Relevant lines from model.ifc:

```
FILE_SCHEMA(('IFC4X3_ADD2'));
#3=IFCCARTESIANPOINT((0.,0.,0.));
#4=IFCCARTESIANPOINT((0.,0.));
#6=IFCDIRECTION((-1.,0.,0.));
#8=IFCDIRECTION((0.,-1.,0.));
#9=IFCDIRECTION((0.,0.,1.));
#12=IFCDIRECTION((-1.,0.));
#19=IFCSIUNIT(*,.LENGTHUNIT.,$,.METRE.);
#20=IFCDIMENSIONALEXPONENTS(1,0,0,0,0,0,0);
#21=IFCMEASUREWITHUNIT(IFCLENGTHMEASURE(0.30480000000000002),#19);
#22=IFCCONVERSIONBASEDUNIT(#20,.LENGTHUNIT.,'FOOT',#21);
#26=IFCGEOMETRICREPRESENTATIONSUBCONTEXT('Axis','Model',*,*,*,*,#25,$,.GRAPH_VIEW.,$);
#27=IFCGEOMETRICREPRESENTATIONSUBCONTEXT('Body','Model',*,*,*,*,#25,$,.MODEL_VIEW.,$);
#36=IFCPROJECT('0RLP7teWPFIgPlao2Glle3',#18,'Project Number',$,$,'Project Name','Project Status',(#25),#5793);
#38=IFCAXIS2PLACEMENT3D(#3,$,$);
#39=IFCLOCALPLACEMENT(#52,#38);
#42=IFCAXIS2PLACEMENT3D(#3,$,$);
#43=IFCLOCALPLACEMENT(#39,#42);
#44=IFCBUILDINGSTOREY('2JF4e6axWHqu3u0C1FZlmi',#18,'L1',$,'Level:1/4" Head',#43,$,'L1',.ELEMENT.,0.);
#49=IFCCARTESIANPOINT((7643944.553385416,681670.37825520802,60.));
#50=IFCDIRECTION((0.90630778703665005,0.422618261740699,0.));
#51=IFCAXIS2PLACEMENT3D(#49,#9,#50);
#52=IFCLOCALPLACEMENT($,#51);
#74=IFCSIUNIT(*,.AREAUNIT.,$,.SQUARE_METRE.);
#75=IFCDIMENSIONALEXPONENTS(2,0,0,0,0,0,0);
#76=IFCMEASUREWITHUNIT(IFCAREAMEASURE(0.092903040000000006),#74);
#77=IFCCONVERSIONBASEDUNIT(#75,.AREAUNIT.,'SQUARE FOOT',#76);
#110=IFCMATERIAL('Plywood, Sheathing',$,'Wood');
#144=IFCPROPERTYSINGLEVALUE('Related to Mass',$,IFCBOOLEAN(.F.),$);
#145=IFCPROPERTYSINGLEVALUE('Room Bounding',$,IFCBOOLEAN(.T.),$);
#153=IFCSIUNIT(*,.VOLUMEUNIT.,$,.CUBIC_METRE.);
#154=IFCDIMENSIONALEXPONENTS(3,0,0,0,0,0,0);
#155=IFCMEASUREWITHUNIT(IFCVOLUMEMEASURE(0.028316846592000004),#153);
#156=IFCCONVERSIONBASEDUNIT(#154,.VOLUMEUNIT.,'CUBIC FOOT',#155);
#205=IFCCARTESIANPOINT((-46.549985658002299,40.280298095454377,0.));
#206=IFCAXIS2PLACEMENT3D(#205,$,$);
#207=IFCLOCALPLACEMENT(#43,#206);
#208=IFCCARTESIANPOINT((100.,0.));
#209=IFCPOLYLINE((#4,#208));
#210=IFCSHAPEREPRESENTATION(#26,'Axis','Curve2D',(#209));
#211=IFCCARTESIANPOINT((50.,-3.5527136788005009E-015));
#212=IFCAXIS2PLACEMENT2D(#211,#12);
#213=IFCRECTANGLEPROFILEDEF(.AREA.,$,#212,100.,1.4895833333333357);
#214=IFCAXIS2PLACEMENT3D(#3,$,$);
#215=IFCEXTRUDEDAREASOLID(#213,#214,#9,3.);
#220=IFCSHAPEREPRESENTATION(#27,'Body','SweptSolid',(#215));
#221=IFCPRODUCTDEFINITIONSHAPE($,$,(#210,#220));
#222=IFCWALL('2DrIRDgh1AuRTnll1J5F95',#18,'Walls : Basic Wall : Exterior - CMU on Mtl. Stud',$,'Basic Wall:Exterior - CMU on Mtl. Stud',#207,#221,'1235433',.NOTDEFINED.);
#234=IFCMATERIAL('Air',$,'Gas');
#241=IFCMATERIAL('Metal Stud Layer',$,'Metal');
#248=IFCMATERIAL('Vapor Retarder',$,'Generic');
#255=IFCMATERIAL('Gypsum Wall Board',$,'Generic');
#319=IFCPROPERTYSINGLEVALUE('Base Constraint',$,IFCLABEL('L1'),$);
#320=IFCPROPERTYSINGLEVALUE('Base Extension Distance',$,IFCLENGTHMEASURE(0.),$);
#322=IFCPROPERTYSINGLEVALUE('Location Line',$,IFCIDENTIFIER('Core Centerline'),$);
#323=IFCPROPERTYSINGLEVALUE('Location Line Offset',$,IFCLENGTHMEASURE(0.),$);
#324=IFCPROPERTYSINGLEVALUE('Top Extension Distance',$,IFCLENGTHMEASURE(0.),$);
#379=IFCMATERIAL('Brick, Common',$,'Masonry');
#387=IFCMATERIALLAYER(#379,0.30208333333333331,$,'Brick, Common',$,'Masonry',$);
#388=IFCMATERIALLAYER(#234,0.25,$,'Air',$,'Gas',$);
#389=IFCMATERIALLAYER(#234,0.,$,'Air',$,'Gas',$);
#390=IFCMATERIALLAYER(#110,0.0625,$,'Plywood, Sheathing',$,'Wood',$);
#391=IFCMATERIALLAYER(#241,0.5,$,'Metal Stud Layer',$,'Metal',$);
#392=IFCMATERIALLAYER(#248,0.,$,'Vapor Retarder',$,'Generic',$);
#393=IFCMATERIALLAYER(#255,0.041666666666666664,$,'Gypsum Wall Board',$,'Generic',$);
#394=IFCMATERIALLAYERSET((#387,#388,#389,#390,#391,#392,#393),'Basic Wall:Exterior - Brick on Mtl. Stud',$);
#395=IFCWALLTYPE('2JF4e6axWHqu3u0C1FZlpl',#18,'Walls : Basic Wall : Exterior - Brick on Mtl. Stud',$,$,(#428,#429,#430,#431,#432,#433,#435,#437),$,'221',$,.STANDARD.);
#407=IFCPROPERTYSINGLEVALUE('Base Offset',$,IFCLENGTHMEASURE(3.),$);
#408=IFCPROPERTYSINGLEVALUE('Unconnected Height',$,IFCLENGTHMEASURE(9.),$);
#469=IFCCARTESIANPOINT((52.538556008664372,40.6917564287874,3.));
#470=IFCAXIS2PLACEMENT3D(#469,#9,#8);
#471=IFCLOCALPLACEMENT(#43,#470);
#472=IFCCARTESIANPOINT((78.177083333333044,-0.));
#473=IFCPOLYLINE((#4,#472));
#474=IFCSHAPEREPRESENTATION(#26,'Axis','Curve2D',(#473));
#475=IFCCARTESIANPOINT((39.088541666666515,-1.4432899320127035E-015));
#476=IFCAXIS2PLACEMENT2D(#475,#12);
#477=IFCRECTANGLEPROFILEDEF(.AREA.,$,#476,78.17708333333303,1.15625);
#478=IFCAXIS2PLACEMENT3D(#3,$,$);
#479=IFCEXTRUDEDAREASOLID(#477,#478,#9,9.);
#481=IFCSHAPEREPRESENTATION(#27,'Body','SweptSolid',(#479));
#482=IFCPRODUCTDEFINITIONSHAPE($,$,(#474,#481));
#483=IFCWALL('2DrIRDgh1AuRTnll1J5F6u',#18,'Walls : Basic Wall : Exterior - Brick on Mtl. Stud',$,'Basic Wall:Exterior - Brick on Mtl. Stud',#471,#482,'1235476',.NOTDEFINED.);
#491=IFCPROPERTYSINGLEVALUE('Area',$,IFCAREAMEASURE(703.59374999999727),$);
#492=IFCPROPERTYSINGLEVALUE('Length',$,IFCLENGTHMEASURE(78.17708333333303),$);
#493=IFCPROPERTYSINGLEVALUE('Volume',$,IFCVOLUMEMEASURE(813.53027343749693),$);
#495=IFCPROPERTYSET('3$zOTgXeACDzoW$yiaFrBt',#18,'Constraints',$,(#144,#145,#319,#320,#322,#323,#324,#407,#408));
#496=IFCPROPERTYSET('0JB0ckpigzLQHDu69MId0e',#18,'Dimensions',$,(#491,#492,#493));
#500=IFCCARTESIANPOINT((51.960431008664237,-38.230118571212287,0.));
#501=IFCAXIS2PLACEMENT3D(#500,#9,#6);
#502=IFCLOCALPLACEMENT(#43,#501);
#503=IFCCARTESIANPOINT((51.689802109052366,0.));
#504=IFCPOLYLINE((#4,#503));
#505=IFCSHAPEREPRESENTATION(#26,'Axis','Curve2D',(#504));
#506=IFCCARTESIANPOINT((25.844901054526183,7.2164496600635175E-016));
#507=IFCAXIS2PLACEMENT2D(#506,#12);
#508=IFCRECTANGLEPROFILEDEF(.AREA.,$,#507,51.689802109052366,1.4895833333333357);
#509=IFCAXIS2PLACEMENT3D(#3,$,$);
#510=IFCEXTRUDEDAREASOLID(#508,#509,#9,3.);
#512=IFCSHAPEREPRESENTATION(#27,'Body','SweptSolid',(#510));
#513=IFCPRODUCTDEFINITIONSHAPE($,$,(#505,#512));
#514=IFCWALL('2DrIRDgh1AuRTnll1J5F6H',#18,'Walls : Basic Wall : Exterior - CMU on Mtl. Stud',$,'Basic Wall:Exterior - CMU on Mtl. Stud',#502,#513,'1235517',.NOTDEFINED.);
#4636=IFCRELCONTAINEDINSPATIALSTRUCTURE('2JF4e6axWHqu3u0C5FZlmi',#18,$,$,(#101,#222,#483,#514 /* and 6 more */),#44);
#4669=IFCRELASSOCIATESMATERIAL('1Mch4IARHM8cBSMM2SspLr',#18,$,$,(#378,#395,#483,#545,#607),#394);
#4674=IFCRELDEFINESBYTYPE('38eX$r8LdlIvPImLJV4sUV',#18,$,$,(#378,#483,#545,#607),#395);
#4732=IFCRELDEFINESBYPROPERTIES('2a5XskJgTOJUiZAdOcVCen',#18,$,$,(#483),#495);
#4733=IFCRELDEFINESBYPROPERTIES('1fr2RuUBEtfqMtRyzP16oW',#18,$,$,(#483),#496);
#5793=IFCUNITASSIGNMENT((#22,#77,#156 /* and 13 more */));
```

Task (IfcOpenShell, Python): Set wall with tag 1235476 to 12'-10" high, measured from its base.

```python
import ifcopenshell
import ifcopenshell.api.pset
import ifcopenshell.geom
import ifcopenshell.util.element
import ifcopenshell.util.representation
import ifcopenshell.util.shape
import ifcopenshell.util.unit

model = ifcopenshell.open("model.ifc")
unit_scale = ifcopenshell.util.unit.calculate_unit_scale(model)
area_scale = ifcopenshell.util.unit.calculate_unit_scale(model, "AREAUNIT")
volume_scale = ifcopenshell.util.unit.calculate_unit_scale(model, "VOLUMEUNIT")
settings = ifcopenshell.geom.settings()


def volume(element):
    """Net volume in cubic metres, openings subtracted."""
    shape = ifcopenshell.geom.create_shape(settings, element)
    return ifcopenshell.util.shape.get_volume(shape.geometry)


wall = model.by_id(483)
before = volume(wall)

body = ifcopenshell.util.representation.get_representation(wall, "Model", "Body")
solid = body.Items[0]
old_height = solid.Depth
solid.Depth = 154 * 0.0254 / unit_scale
after = volume(wall)
thickness = 0.3524  # wall thickness in metres

# Update the stored height, areas and volumes.
pset = model.by_id(ifcopenshell.util.element.get_pset(wall, "Constraints", should_inherit=False)["id"])
ifcopenshell.api.pset.edit_pset(model, pset=pset, properties={
    "Unconnected Height": model.create_entity("IfcLengthMeasure", solid.Depth),
})
pset = model.by_id(ifcopenshell.util.element.get_pset(wall, "Dimensions", should_inherit=False)["id"])
ifcopenshell.api.pset.edit_pset(model, pset=pset, properties={
    "Area": model.create_entity("IfcAreaMeasure", after / thickness / area_scale),
    "Volume": model.create_entity("IfcVolumeMeasure", after / volume_scale),
})

print(f"height {old_height:g} -> {solid.Depth:g}, volume {before:.3f} -> {after:.3f} m3")

model.write("model_updated.ifc")
```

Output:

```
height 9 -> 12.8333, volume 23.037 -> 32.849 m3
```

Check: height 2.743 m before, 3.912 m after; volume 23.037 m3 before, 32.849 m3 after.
